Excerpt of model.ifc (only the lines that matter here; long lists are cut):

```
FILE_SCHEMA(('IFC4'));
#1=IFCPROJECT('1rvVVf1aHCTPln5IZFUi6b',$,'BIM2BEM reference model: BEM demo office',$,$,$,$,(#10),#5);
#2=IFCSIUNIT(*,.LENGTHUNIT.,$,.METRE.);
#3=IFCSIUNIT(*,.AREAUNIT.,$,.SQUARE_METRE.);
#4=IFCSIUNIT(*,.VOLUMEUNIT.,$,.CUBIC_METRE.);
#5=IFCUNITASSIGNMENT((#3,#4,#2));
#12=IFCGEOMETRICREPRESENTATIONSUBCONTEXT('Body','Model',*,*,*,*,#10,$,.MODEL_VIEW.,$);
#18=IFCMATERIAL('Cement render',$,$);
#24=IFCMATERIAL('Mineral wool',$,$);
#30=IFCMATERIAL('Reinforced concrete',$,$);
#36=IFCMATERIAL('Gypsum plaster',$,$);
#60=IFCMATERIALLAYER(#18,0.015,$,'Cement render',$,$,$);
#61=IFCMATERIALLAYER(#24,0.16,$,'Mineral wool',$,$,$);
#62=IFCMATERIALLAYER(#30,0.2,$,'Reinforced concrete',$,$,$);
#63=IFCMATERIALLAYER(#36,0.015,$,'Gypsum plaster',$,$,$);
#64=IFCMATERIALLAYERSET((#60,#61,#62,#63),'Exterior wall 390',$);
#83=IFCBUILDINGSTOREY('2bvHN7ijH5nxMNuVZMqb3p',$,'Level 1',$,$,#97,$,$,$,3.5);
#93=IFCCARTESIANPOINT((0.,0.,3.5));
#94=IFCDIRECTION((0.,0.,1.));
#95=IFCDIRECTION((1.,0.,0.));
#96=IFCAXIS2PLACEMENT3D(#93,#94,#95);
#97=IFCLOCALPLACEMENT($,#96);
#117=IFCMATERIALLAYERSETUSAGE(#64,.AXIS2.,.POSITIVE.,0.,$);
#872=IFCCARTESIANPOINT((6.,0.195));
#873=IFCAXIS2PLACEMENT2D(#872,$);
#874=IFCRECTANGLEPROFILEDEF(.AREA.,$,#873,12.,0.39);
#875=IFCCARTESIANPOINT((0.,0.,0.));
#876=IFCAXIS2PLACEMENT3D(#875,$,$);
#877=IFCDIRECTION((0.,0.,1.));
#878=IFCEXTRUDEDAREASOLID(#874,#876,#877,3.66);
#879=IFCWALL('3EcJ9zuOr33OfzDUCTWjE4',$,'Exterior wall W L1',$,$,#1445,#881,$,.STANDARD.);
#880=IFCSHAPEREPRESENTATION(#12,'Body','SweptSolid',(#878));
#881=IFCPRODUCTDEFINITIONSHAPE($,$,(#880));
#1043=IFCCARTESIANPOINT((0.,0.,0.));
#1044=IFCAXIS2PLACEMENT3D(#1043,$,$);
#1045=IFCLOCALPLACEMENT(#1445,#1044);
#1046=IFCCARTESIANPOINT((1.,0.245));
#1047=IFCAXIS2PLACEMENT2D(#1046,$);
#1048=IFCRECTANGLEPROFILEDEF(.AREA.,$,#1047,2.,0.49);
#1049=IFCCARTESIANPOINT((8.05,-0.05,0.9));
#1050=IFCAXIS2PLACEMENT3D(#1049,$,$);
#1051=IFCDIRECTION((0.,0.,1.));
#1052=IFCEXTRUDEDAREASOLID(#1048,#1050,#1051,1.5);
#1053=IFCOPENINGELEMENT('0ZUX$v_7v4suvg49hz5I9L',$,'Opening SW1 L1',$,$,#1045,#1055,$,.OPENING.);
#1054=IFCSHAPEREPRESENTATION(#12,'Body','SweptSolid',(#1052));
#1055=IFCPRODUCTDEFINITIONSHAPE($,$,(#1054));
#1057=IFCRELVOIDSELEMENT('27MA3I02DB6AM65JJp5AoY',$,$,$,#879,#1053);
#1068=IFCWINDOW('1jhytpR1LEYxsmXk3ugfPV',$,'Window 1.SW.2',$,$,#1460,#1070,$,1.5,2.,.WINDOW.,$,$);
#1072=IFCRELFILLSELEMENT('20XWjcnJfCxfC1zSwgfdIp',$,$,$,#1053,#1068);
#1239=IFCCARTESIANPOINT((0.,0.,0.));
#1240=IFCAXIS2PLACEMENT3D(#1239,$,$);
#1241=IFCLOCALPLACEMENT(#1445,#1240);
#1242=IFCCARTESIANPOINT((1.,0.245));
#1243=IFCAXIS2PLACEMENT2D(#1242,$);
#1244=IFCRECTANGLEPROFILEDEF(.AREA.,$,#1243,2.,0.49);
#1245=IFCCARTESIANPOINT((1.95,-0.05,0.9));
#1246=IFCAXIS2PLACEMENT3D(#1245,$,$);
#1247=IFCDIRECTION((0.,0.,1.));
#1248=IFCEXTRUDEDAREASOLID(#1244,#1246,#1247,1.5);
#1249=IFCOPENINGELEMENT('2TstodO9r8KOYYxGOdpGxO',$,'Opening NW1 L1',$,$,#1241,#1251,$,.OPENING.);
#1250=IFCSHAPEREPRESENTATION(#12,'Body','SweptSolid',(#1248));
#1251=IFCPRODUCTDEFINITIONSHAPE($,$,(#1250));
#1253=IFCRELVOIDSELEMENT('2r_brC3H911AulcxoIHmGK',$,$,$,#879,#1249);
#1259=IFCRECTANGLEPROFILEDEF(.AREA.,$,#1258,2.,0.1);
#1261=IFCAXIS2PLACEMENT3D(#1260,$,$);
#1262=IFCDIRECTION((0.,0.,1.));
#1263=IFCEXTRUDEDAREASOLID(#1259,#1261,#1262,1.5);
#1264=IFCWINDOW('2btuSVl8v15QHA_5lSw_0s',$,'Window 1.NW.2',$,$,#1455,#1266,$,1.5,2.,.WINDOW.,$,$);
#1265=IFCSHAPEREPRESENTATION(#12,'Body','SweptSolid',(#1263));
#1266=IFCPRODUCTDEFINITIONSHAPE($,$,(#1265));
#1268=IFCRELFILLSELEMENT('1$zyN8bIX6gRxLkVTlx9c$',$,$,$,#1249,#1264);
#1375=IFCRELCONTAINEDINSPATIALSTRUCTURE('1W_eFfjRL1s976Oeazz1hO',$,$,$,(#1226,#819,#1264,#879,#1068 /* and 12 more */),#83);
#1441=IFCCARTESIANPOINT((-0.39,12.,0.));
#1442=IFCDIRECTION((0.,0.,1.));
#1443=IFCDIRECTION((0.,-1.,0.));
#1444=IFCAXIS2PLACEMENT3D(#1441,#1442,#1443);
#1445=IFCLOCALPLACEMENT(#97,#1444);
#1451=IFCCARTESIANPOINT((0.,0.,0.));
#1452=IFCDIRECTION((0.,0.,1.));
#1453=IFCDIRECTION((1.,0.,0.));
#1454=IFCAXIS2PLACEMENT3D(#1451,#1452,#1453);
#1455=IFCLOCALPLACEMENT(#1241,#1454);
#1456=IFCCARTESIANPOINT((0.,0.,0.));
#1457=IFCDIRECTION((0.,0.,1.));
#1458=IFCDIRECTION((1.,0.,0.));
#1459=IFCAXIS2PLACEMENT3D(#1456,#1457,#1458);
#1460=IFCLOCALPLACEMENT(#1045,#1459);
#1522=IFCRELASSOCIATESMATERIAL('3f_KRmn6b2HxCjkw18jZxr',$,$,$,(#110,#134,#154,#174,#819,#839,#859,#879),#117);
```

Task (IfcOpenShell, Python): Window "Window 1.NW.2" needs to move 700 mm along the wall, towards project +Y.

```python
import ifcopenshell
import ifcopenshell.api.geometry
import ifcopenshell.util.placement

model = ifcopenshell.open("model.ifc")

window = model.by_id(1264)
opening = window.FillsVoids[0].RelatingOpeningElement
wall = opening.VoidsElements[0].RelatingBuildingElement

wall_matrix = ifcopenshell.util.placement.get_local_placement(wall.ObjectPlacement)
shift = wall_matrix[:3, 0] * -0.7
before = ifcopenshell.util.placement.get_local_placement(window.ObjectPlacement)[:3, 3].copy()

# The window is placed relative to its opening, so it follows when the opening moves.
matrix = ifcopenshell.util.placement.get_local_placement(opening.ObjectPlacement)
matrix[:3, 3] += shift
ifcopenshell.api.geometry.edit_object_placement(
    model, product=opening, matrix=matrix, is_si=False, should_transform_children=True
)

after = ifcopenshell.util.placement.get_local_placement(window.ObjectPlacement)[:3, 3]
print("window moved by", (after - before).round(3) + 0.0)

model.write("model_updated.ifc")
```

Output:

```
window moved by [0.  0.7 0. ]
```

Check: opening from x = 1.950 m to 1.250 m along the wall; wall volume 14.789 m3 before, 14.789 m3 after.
